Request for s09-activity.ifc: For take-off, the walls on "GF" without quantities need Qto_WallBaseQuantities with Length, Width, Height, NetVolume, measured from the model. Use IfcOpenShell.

First a look at what the model holds.

```python
import ifcopenshell
import ifcopenshell.util.element
import ifcopenshell.util.unit

model = ifcopenshell.open("s09-activity.ifc")
print(model.schema)
for unit_type in ("LENGTHUNIT", "AREAUNIT", "VOLUMEUNIT"):
    print(unit_type, ifcopenshell.util.unit.calculate_unit_scale(model, unit_type))
storey = next(s for s in model.by_type("IfcBuildingStorey") if s.Name == "GF")
walls = [e for e in ifcopenshell.util.element.get_decomposition(storey) if e.is_a("IfcWall")]
for e in sorted(walls, key=lambda e: e.id()):
    print(e.id(), e.is_a(), e.Name, list(ifcopenshell.util.element.get_psets(e, qtos_only=True)), sep=" | ")
```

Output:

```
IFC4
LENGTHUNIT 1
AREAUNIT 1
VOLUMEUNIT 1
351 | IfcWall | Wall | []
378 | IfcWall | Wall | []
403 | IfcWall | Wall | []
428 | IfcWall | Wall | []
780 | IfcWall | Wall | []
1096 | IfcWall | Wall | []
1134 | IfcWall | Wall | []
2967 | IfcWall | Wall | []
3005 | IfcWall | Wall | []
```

```python
import ifcopenshell
import ifcopenshell.api.pset
import ifcopenshell.geom
import ifcopenshell.util.element
import ifcopenshell.util.shape
import ifcopenshell.util.unit

model = ifcopenshell.open("s09-activity.ifc")
unit_scale = ifcopenshell.util.unit.calculate_unit_scale(model)
volume_scale = ifcopenshell.util.unit.calculate_unit_scale(model, "VOLUMEUNIT")
settings = ifcopenshell.geom.settings()

storey = next(s for s in model.by_type("IfcBuildingStorey") if s.Name == "GF")
walls = [e for e in ifcopenshell.util.element.get_decomposition(storey) if e.is_a("IfcWall")]

for e in sorted(walls, key=lambda e: e.id()):
    if ifcopenshell.util.element.get_psets(e, qtos_only=True, should_inherit=False):
        continue
    # Geometry comes back in metres, in the element's own axes.
    shape = ifcopenshell.geom.create_shape(settings, e)
    values = {
        "Length": ifcopenshell.util.shape.get_x(shape.geometry) / unit_scale,
        "Width": ifcopenshell.util.shape.get_y(shape.geometry) / unit_scale,
        "Height": ifcopenshell.util.shape.get_z(shape.geometry) / unit_scale,
        "NetVolume": ifcopenshell.util.shape.get_volume(shape.geometry) / volume_scale,
    }
    qto = ifcopenshell.api.pset.add_qto(model, product=e, name="Qto_WallBaseQuantities")
    ifcopenshell.api.pset.edit_qto(model, qto=qto, properties=values)
    print(e.id(), {k: round(v, 3) for k, v in values.items()})

model.write("s09-activity_updated.ifc")
```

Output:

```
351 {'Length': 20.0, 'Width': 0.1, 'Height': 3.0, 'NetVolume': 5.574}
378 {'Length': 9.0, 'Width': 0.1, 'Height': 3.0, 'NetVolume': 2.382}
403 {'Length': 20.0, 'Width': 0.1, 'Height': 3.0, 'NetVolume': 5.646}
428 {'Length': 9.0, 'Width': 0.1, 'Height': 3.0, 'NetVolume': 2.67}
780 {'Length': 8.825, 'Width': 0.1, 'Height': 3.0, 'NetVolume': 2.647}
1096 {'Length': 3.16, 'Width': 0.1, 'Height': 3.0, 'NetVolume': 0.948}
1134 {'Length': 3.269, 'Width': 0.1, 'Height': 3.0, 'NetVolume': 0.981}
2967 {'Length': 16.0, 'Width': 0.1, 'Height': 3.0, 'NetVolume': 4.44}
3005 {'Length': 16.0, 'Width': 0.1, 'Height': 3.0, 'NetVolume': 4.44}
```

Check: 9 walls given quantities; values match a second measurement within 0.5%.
